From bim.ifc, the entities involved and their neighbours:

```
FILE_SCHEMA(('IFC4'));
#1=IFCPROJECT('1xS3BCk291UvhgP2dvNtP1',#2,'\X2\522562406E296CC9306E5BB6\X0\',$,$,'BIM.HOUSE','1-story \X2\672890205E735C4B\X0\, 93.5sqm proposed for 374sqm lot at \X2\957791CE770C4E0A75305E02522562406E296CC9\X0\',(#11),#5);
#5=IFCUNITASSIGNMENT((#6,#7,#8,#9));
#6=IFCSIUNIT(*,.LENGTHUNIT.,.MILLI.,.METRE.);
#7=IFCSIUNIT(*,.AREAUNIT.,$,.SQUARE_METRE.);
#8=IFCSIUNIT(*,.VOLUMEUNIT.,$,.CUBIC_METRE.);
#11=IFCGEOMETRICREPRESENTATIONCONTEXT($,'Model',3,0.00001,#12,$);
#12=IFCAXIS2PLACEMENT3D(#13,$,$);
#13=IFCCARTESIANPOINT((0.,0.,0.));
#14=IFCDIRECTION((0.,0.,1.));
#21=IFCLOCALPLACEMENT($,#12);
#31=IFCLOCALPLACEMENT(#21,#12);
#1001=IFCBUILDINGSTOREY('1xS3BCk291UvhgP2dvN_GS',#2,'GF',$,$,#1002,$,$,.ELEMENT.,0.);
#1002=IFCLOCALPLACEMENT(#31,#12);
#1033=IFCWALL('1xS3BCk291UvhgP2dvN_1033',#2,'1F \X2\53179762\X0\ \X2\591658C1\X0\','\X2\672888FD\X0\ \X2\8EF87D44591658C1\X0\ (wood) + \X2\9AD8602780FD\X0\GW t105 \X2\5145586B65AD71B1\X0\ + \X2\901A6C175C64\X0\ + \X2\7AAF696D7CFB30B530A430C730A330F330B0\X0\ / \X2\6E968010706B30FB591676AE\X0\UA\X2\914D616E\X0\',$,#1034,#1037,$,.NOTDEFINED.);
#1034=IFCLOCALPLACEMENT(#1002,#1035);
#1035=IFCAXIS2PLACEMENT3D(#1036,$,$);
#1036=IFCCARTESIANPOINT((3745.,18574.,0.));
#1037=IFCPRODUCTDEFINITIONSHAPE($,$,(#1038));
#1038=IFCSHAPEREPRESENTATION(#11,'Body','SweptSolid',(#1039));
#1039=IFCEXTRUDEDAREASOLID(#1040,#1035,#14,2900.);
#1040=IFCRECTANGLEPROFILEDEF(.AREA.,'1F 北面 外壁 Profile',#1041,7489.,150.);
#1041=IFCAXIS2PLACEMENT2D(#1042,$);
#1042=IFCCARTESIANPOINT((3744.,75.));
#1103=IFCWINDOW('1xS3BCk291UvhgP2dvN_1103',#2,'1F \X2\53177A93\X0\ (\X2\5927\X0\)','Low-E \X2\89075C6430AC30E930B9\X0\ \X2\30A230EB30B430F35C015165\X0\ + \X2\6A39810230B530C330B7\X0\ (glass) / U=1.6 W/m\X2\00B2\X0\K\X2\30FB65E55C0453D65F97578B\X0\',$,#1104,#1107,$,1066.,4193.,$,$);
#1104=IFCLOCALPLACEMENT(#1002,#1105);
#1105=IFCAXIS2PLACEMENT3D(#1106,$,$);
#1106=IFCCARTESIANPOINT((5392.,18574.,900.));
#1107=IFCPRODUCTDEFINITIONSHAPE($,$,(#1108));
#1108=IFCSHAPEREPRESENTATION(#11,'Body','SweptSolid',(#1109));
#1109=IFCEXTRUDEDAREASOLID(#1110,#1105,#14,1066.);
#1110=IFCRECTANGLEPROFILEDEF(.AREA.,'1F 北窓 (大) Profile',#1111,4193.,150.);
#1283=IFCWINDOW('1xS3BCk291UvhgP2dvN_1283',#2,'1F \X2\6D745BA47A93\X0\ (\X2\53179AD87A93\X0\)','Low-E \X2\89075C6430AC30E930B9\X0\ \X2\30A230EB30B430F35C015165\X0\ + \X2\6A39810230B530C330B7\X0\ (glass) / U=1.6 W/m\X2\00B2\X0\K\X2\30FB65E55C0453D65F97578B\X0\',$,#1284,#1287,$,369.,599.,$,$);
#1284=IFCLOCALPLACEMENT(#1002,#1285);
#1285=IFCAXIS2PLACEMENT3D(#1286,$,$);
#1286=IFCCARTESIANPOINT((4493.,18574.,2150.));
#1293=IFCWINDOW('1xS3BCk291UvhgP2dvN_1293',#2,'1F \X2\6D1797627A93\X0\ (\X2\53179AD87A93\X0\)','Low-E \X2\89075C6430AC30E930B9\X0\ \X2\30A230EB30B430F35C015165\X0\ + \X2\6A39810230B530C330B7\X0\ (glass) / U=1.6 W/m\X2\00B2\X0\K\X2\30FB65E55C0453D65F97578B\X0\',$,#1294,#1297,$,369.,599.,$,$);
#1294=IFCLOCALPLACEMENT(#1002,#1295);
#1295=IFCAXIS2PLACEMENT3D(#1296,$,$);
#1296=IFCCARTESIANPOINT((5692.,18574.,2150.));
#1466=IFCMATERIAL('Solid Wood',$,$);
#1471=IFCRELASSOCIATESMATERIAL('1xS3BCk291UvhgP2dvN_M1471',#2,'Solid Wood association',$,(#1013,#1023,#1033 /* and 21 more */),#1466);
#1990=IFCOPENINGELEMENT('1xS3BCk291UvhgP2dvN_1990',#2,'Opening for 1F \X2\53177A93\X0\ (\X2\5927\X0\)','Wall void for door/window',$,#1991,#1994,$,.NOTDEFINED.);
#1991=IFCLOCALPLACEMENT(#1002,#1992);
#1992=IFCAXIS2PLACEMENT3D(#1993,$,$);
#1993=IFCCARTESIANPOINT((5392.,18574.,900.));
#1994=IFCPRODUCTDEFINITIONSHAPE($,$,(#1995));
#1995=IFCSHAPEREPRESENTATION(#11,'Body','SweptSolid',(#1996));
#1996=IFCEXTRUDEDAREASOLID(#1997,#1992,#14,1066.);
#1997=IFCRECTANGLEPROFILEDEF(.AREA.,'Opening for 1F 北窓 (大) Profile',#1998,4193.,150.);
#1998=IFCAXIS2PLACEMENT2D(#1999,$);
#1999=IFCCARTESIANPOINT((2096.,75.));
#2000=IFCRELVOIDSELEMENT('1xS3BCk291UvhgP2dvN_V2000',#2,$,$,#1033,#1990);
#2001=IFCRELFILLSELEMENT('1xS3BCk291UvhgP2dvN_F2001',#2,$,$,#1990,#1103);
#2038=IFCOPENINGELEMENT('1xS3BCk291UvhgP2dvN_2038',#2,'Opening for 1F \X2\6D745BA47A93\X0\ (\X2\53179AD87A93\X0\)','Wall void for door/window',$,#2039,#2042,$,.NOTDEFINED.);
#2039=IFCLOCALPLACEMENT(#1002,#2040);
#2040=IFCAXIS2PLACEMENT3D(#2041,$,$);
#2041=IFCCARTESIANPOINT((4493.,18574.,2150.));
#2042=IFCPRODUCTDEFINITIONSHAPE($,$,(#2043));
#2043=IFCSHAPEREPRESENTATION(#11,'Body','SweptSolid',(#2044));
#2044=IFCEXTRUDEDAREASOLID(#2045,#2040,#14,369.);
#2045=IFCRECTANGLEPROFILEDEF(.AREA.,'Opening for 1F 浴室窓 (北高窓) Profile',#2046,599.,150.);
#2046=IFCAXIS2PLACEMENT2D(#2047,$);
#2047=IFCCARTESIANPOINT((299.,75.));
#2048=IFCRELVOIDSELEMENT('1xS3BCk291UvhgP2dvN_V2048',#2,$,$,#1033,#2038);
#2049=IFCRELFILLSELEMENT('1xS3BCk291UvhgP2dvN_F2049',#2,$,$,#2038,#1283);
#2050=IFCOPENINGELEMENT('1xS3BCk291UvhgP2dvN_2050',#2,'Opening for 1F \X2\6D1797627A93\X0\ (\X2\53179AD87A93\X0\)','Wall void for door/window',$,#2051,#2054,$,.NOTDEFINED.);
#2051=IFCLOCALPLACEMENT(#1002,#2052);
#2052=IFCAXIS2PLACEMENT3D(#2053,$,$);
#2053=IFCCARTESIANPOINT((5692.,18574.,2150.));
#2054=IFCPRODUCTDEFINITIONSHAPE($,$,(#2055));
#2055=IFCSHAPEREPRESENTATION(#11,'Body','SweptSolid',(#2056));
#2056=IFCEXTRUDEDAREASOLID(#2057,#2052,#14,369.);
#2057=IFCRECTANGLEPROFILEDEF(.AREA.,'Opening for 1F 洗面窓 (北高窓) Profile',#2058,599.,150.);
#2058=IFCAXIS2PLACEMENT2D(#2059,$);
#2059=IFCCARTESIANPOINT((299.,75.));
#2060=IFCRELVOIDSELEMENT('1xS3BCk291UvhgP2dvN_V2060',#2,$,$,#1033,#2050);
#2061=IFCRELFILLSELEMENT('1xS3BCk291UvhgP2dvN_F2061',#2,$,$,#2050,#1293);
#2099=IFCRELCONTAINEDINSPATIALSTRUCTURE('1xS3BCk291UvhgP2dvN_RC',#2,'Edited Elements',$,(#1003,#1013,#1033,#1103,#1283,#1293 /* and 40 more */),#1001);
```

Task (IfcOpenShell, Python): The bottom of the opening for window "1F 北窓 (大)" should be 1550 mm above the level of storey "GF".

```python
import numpy as np
import ifcopenshell
import ifcopenshell.api.geometry
import ifcopenshell.geom
import ifcopenshell.util.element
import ifcopenshell.util.placement
import ifcopenshell.util.shape
import ifcopenshell.util.unit

model = ifcopenshell.open("bim.ifc")
unit_scale = ifcopenshell.util.unit.calculate_unit_scale(model)

window = model.by_guid("1xS3BCk291UvhgP2dvN_1103")
opening = window.FillsVoids[0].RelatingOpeningElement
storey = ifcopenshell.util.element.get_container(window, ifc_class="IfcBuildingStorey")
level = ifcopenshell.util.placement.get_local_placement(storey.ObjectPlacement)[2, 3]

# The opening's origin need not be at the sill, so measure its lowest point.
shape = ifcopenshell.geom.create_shape(ifcopenshell.geom.settings(), opening)
bottom = ifcopenshell.util.shape.get_shape_bottom_elevation(shape, shape.geometry) / unit_scale
dz = level + 1.55 / unit_scale - bottom

shift = np.array([0.0, 0.0, dz])
# The window is not placed relative to its opening, so move both.
for product in (opening, window):
    matrix = ifcopenshell.util.placement.get_local_placement(product.ObjectPlacement)
    matrix[:3, 3] += shift
    ifcopenshell.api.geometry.edit_object_placement(model, product=product, matrix=matrix, is_si=False)

print(f"moved by {dz * unit_scale:+.3f} m")

model.write("bim_v2.ifc")
```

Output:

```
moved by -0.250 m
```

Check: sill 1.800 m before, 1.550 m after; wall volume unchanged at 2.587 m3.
